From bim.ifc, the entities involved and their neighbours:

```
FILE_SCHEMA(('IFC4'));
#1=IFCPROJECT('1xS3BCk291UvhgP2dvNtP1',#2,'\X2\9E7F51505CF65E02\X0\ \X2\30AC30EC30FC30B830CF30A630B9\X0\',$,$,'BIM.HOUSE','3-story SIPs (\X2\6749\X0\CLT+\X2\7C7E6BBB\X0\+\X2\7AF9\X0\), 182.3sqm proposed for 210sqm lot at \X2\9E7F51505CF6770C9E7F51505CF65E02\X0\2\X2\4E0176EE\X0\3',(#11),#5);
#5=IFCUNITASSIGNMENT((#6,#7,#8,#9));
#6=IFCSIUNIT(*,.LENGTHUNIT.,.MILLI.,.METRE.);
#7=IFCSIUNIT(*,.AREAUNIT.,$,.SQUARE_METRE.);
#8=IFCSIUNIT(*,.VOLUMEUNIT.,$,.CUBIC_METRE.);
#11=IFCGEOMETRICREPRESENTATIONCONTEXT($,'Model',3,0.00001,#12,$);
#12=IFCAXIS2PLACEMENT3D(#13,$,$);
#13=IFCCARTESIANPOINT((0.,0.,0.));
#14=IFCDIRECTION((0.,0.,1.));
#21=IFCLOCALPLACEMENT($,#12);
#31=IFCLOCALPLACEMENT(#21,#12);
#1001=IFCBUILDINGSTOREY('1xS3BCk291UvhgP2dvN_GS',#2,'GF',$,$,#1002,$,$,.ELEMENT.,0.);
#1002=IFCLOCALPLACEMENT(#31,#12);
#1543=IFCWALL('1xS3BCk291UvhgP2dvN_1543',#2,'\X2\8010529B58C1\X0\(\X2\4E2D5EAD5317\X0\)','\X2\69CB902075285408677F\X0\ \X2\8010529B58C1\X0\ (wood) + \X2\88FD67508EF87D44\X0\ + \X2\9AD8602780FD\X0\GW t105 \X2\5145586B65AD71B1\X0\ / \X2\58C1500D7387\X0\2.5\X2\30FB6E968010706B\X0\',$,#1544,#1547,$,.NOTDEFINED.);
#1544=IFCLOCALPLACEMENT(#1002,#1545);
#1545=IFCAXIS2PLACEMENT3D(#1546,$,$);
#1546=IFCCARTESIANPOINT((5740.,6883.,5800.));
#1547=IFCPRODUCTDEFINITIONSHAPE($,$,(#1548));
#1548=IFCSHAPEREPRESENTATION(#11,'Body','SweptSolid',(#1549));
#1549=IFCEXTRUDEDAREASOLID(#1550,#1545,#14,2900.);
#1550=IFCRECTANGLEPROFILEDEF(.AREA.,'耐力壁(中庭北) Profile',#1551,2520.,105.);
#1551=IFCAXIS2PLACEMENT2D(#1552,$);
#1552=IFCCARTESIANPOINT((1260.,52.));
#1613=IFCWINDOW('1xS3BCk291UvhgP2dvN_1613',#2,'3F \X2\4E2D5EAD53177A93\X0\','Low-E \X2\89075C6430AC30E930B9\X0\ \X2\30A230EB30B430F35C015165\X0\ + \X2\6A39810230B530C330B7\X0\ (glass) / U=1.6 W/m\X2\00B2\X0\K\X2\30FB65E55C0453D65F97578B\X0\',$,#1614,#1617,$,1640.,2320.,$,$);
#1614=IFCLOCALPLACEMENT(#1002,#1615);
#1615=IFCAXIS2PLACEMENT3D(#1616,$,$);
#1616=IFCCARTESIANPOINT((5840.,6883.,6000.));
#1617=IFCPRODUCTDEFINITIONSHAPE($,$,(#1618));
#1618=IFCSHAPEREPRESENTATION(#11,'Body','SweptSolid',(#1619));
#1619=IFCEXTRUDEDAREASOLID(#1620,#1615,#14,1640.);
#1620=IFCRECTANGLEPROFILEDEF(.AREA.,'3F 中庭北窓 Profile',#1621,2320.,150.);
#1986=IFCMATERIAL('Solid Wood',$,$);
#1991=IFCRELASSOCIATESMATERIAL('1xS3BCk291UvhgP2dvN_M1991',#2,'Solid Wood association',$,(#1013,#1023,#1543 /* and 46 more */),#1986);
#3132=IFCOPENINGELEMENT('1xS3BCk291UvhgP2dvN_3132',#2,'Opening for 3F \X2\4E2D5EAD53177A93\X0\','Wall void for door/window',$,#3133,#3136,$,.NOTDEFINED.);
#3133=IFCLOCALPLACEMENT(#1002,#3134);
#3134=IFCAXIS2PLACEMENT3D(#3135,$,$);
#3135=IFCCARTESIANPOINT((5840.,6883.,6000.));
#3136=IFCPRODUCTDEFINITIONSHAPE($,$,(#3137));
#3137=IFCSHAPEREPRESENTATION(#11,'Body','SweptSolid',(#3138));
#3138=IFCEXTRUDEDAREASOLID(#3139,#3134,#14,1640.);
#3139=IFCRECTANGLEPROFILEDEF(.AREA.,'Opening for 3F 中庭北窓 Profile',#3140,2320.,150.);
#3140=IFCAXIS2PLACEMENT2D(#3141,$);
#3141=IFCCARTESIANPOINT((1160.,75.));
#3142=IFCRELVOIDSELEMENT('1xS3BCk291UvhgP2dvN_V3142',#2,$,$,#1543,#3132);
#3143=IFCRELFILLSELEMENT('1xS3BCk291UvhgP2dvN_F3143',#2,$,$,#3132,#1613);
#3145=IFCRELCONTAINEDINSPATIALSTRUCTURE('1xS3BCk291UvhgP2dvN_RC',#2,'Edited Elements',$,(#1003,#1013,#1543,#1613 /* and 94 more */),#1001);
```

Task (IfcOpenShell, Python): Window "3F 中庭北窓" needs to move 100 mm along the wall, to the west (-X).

```python
import ifcopenshell
import ifcopenshell.api.geometry
import ifcopenshell.util.placement
import ifcopenshell.util.unit

model = ifcopenshell.open("bim.ifc")
unit_scale = ifcopenshell.util.unit.calculate_unit_scale(model)

window = model.by_id(1613)
opening = window.FillsVoids[0].RelatingOpeningElement
wall = opening.VoidsElements[0].RelatingBuildingElement

wall_matrix = ifcopenshell.util.placement.get_local_placement(wall.ObjectPlacement)
shift = wall_matrix[:3, 0] * -0.1 / unit_scale
before = ifcopenshell.util.placement.get_local_placement(window.ObjectPlacement)[:3, 3].copy()

# The window is not placed relative to its opening, so move both.
for product in (opening, window):
    matrix = ifcopenshell.util.placement.get_local_placement(product.ObjectPlacement)
    matrix[:3, 3] += shift
    ifcopenshell.api.geometry.edit_object_placement(model, product=product, matrix=matrix, is_si=False)

after = ifcopenshell.util.placement.get_local_placement(window.ObjectPlacement)[:3, 3]
print("window moved by", (after - before).round(3) + 0.0)

model.write("bim_rev.ifc")
```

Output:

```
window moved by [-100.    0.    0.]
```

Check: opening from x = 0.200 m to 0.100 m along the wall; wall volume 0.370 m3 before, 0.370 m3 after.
